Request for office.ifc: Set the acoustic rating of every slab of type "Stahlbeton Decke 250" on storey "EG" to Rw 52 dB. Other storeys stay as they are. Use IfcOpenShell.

First a look at what the model holds.

```python
import ifcopenshell
import ifcopenshell.util.element

model = ifcopenshell.open("office.ifc")
print(model.schema)
storey = next(s for s in model.by_type("IfcBuildingStorey") if s.Name == "EG")
slabs = [e for e in ifcopenshell.util.element.get_decomposition(storey) if e.is_a("IfcSlab")]
seen = {}
for e in slabs:
    element_type = ifcopenshell.util.element.get_type(e)
    key = (element_type.Name if element_type != e and element_type else None, ifcopenshell.util.element.get_pset(e, "Pset_SlabCommon", "AcousticRating"))
    seen[key] = seen.get(key, 0) + 1
for (name, value), count in sorted(seen.items(), key=str):
    print(count, "x", name, "|", value)
```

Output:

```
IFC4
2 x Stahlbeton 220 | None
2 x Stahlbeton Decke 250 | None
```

```python
import ifcopenshell
import ifcopenshell.api.pset
import ifcopenshell.util.element

model = ifcopenshell.open("office.ifc")

storey = next(s for s in model.by_type("IfcBuildingStorey") if s.Name == "EG")
slabs = [e for e in ifcopenshell.util.element.get_decomposition(storey) if e.is_a("IfcSlab")]

count = 0
for e in slabs:
    element_type = ifcopenshell.util.element.get_type(e)
    if element_type in (None, e) or element_type.Name != "Stahlbeton Decke 250":
        continue
    # add_pset returns the element's existing set when there is one.
    pset = ifcopenshell.api.pset.add_pset(model, product=e, name="Pset_SlabCommon")
    ifcopenshell.api.pset.edit_pset(model, pset=pset, properties={"AcousticRating": "Rw 52 dB"})
    count += 1

print(count, "slabs updated")

model.write("office_v2.ifc")
```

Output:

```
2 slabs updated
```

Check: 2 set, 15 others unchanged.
